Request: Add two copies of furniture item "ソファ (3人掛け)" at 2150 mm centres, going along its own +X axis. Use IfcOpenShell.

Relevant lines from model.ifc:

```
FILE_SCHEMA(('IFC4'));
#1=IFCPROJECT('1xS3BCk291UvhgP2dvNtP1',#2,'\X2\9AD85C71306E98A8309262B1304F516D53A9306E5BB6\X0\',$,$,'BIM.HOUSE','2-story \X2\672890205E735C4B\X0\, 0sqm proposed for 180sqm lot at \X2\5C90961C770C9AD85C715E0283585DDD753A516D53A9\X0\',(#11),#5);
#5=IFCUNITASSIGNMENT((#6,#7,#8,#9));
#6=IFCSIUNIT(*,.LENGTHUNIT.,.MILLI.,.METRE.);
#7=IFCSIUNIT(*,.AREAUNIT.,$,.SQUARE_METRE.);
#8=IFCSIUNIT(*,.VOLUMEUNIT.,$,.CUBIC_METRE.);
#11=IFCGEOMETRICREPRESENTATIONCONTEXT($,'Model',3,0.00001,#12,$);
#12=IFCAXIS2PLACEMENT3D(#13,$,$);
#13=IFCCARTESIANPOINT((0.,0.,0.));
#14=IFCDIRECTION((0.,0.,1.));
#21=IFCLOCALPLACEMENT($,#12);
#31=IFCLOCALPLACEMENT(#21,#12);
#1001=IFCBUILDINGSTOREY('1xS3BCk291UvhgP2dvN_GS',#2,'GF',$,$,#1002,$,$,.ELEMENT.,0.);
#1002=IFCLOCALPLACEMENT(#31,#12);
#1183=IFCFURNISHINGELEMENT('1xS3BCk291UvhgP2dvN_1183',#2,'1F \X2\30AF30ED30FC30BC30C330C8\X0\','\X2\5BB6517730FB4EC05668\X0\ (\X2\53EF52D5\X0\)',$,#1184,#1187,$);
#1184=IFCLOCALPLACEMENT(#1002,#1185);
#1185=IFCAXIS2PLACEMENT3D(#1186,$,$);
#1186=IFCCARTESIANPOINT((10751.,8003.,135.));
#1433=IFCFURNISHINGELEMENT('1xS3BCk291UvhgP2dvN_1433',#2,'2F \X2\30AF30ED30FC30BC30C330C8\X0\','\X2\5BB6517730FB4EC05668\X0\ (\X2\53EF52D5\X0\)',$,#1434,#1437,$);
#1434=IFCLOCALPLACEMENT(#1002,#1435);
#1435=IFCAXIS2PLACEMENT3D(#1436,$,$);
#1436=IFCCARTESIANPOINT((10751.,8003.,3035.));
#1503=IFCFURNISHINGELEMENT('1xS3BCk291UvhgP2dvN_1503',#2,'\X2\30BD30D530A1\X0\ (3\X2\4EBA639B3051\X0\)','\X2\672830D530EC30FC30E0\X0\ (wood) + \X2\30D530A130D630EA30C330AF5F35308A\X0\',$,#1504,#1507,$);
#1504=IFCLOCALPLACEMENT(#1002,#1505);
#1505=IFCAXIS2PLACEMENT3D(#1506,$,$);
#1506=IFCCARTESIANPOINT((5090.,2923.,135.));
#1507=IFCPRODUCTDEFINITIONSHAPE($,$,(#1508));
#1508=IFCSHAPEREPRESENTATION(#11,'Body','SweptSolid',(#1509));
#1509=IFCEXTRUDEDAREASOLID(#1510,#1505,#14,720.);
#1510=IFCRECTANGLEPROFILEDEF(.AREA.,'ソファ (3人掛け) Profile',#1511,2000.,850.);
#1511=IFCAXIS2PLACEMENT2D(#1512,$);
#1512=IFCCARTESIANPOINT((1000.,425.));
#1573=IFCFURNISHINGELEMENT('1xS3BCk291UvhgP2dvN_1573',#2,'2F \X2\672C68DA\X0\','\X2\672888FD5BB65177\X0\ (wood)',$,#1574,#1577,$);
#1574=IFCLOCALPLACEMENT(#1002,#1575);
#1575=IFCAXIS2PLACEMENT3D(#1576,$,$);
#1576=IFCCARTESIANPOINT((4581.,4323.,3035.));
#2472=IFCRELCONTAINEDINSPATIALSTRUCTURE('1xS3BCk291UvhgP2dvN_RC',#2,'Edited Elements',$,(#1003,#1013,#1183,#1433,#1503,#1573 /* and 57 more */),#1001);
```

```python
import ifcopenshell
import ifcopenshell.api.geometry
import ifcopenshell.api.root
import ifcopenshell.util.element
import ifcopenshell.util.placement

model = ifcopenshell.open("model.ifc")


def reuse_history(source, copy):
    """copy_class also copies each property set's owner history, people and application; keep the originals."""
    for rel in copy.IsDefinedBy:
        if rel.is_a("IfcRelDefinesByProperties") and (history := rel.RelatingPropertyDefinition.OwnerHistory):
            rel.RelatingPropertyDefinition.OwnerHistory = source.OwnerHistory
            ifcopenshell.util.element.remove_deep2(model, history)


source = model.by_id(1503)
base = ifcopenshell.util.placement.get_local_placement(source.ObjectPlacement)
step = base[:3, 0] * 2150.0

for i in range(1, 3):
    copy = ifcopenshell.api.root.copy_class(model, product=source)
    copy.Representation = ifcopenshell.util.element.copy_deep(
        model, source.Representation, exclude=["IfcGeometricRepresentationContext", "IfcRepresentationMap"]
    )
    reuse_history(source, copy)
    matrix = base.copy()
    matrix[:3, 3] += i * step
    print("added at", matrix[:3, 3].round(3) + 0.0)
    ifcopenshell.api.geometry.edit_object_placement(model, product=copy, matrix=matrix, is_si=False)

model.write("model_updated.ifc")
```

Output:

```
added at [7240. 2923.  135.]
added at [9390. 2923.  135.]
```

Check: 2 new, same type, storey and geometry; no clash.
